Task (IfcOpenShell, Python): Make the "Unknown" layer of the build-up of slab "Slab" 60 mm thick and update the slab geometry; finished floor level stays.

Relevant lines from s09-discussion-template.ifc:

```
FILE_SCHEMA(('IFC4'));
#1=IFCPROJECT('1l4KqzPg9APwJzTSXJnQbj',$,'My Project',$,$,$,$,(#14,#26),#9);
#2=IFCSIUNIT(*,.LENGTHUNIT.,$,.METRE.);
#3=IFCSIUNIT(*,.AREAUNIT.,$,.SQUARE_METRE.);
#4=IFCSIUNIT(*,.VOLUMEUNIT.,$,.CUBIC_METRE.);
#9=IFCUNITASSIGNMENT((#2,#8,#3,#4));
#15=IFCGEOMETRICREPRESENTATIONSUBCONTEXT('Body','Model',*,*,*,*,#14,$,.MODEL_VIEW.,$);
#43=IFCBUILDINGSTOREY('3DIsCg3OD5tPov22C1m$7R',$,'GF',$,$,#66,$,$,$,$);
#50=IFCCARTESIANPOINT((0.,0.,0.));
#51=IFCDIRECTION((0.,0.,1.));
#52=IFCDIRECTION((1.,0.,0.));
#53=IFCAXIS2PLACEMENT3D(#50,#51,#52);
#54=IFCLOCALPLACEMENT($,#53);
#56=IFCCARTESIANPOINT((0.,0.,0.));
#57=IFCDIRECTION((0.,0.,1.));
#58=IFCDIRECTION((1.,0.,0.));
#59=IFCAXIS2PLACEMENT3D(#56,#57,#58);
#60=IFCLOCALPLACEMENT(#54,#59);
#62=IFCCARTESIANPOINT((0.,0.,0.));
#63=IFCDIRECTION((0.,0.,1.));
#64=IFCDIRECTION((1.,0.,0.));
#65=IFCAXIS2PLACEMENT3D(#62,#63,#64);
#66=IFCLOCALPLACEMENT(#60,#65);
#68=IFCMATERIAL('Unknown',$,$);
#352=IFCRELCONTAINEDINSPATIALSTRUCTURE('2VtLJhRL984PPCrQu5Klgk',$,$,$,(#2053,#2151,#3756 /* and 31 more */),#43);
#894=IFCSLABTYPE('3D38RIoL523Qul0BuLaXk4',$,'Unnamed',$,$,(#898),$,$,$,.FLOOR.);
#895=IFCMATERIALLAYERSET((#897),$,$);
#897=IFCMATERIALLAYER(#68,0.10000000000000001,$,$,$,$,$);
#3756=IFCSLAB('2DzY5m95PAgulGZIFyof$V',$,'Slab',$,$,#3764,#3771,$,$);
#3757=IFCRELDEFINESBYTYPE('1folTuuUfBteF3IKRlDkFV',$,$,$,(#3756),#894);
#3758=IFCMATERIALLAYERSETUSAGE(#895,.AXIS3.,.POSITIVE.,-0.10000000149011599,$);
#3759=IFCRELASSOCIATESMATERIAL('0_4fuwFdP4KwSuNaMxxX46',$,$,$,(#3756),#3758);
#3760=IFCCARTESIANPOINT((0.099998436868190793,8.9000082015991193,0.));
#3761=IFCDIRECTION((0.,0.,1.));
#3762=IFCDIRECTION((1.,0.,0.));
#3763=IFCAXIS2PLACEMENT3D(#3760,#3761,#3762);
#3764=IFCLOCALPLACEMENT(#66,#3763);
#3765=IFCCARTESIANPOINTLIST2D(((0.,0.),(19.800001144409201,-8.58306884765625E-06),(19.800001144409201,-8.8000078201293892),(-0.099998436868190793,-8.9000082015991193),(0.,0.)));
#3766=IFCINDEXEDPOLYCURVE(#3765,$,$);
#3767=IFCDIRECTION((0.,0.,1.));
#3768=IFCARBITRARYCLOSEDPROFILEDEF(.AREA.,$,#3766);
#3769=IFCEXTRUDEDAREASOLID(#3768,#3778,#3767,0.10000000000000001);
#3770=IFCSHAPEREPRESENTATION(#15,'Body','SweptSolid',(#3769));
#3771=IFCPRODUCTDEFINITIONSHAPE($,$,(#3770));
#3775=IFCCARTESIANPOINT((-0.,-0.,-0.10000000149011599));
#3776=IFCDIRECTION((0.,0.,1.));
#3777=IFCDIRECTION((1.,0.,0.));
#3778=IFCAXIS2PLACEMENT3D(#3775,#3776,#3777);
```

```python
import ifcopenshell
import ifcopenshell.util.element
import ifcopenshell.util.representation

model = ifcopenshell.open("s09-discussion-template.ifc")

layer_set = model.by_id(895)
layer = next(l for l in layer_set.MaterialLayers if l.Material and l.Material.Name == "Unknown")
change = 0.06 - layer.LayerThickness
layer.LayerThickness += change

# Geometry does not follow the layer set by itself.
slabs = [e for e in ifcopenshell.util.element.get_elements_by_material(model, layer_set) if e.is_a("IfcSlab")]
for slab in sorted(slabs, key=lambda e: e.id()):
    body = ifcopenshell.util.representation.get_representation(slab, "Model", "Body")
    solid = body.Items[0]
    old_depth = solid.Depth
    solid.Depth += change
    # Extruded upwards: lower the start of the extrusion so the top stays.
    x, y, z = solid.Position.Location.Coordinates
    solid.Position.Location = model.createIfcCartesianPoint((x, y, z - change))
    print(slab.id(), f"{old_depth:g} -> {solid.Depth:g}")

# The layers are counted up from the underside, which has moved.
for usage in {ifcopenshell.util.element.get_material(slab) for slab in slabs}:
    usage.OffsetFromReferenceLine -= change

model.write("s09-discussion-template_rev.ifc")
```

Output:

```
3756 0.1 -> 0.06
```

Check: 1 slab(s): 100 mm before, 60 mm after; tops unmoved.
